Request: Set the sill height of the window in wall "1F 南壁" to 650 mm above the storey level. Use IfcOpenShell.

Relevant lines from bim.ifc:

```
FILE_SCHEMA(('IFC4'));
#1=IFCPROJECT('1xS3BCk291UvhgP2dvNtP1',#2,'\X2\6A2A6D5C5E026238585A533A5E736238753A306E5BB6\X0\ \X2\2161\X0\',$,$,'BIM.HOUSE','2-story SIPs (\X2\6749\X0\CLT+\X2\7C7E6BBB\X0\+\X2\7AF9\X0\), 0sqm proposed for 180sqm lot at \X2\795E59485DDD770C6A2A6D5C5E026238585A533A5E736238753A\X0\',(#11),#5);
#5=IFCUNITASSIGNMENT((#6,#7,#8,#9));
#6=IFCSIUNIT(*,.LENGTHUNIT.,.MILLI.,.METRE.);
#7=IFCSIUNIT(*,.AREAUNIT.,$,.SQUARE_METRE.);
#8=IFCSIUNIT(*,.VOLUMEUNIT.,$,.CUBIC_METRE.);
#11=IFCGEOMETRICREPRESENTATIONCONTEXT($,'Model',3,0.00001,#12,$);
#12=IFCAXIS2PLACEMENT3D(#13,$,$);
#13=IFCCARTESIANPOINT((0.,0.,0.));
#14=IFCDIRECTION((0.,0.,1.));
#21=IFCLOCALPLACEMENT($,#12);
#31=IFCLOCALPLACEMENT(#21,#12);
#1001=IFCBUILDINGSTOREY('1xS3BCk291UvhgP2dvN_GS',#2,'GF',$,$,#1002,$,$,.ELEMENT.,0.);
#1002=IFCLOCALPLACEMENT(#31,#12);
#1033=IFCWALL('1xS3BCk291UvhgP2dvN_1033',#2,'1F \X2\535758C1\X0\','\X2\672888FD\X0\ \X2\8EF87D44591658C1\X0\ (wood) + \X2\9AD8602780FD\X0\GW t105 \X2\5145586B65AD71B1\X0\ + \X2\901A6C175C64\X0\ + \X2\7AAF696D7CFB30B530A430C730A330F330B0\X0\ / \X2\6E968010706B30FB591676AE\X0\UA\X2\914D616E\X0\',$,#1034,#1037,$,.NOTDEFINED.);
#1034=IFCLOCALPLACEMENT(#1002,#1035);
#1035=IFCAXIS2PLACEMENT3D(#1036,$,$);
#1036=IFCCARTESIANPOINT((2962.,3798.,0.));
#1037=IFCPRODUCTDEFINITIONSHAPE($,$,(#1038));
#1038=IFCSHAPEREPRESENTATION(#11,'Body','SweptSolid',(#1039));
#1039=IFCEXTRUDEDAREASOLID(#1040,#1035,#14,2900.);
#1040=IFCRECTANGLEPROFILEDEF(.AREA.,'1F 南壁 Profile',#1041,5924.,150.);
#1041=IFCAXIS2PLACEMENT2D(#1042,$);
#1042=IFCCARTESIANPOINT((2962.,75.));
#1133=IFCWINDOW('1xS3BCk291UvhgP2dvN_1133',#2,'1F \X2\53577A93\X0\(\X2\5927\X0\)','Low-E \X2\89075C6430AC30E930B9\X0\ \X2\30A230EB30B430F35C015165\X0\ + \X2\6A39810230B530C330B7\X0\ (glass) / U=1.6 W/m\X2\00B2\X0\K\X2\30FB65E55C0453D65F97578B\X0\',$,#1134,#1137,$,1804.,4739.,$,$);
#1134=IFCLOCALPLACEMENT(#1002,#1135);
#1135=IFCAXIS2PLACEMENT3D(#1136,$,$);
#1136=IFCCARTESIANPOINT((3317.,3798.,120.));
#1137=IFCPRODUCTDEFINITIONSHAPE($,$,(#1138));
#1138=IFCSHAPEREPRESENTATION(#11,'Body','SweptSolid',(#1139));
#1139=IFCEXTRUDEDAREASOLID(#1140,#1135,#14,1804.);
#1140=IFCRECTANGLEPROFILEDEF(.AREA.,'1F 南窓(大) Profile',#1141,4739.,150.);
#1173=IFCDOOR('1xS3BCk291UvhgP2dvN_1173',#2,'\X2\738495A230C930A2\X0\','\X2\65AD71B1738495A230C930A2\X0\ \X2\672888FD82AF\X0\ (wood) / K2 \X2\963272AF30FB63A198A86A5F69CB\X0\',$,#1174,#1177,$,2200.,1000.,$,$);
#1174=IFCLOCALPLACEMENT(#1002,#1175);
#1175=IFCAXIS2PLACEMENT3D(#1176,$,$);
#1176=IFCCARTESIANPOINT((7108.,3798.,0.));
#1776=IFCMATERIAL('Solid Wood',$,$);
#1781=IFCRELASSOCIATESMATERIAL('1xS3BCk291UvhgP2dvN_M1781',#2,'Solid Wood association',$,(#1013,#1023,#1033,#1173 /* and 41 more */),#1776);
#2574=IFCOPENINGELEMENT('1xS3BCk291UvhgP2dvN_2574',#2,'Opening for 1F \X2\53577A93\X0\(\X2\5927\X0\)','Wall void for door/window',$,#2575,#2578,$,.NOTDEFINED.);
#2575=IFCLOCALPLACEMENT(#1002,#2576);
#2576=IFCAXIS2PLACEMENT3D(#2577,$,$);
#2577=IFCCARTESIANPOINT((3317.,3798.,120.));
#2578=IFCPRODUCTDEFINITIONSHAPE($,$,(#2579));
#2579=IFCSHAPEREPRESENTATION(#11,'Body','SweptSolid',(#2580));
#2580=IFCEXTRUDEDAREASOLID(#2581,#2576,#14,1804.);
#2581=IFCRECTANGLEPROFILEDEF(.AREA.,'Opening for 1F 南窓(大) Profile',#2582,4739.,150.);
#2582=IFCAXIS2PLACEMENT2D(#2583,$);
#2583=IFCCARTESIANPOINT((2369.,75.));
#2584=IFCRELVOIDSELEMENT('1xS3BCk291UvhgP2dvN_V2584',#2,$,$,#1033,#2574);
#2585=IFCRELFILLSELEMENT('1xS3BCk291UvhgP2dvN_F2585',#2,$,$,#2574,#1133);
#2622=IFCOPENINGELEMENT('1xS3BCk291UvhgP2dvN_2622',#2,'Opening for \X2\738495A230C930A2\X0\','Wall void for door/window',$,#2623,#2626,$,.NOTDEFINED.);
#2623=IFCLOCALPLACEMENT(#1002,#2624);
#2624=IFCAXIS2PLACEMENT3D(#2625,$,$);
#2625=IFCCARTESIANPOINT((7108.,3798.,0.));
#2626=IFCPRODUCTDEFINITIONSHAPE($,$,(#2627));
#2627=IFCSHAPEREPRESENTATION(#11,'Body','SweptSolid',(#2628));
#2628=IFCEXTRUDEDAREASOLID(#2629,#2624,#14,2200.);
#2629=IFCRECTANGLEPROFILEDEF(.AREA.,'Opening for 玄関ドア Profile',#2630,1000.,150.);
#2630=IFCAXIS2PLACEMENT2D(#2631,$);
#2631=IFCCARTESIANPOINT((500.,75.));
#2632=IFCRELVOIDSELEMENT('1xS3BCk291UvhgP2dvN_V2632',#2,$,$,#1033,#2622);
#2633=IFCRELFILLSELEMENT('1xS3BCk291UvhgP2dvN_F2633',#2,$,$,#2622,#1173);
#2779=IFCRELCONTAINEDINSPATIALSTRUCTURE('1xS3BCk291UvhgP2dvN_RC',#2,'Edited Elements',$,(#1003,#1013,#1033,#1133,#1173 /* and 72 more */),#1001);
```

```python
import numpy as np
import ifcopenshell
import ifcopenshell.api.geometry
import ifcopenshell.geom
import ifcopenshell.util.element
import ifcopenshell.util.placement
import ifcopenshell.util.shape
import ifcopenshell.util.unit

model = ifcopenshell.open("bim.ifc")
unit_scale = ifcopenshell.util.unit.calculate_unit_scale(model)

window = model.by_guid("1xS3BCk291UvhgP2dvN_1133")
opening = window.FillsVoids[0].RelatingOpeningElement
storey = ifcopenshell.util.element.get_container(window, ifc_class="IfcBuildingStorey")
level = ifcopenshell.util.placement.get_local_placement(storey.ObjectPlacement)[2, 3]

# The opening's origin need not be at the sill, so measure its lowest point.
shape = ifcopenshell.geom.create_shape(ifcopenshell.geom.settings(), opening)
bottom = ifcopenshell.util.shape.get_shape_bottom_elevation(shape, shape.geometry) / unit_scale
dz = level + 650.0 - bottom

shift = np.array([0.0, 0.0, dz])
# The window is not placed relative to its opening, so move both.
for product in (opening, window):
    matrix = ifcopenshell.util.placement.get_local_placement(product.ObjectPlacement)
    matrix[:3, 3] += shift
    ifcopenshell.api.geometry.edit_object_placement(model, product=product, matrix=matrix, is_si=False)

print(f"moved by {dz * unit_scale:+.3f} m")

model.write("bim_v2.ifc")
```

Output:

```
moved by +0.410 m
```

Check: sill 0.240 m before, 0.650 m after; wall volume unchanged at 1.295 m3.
